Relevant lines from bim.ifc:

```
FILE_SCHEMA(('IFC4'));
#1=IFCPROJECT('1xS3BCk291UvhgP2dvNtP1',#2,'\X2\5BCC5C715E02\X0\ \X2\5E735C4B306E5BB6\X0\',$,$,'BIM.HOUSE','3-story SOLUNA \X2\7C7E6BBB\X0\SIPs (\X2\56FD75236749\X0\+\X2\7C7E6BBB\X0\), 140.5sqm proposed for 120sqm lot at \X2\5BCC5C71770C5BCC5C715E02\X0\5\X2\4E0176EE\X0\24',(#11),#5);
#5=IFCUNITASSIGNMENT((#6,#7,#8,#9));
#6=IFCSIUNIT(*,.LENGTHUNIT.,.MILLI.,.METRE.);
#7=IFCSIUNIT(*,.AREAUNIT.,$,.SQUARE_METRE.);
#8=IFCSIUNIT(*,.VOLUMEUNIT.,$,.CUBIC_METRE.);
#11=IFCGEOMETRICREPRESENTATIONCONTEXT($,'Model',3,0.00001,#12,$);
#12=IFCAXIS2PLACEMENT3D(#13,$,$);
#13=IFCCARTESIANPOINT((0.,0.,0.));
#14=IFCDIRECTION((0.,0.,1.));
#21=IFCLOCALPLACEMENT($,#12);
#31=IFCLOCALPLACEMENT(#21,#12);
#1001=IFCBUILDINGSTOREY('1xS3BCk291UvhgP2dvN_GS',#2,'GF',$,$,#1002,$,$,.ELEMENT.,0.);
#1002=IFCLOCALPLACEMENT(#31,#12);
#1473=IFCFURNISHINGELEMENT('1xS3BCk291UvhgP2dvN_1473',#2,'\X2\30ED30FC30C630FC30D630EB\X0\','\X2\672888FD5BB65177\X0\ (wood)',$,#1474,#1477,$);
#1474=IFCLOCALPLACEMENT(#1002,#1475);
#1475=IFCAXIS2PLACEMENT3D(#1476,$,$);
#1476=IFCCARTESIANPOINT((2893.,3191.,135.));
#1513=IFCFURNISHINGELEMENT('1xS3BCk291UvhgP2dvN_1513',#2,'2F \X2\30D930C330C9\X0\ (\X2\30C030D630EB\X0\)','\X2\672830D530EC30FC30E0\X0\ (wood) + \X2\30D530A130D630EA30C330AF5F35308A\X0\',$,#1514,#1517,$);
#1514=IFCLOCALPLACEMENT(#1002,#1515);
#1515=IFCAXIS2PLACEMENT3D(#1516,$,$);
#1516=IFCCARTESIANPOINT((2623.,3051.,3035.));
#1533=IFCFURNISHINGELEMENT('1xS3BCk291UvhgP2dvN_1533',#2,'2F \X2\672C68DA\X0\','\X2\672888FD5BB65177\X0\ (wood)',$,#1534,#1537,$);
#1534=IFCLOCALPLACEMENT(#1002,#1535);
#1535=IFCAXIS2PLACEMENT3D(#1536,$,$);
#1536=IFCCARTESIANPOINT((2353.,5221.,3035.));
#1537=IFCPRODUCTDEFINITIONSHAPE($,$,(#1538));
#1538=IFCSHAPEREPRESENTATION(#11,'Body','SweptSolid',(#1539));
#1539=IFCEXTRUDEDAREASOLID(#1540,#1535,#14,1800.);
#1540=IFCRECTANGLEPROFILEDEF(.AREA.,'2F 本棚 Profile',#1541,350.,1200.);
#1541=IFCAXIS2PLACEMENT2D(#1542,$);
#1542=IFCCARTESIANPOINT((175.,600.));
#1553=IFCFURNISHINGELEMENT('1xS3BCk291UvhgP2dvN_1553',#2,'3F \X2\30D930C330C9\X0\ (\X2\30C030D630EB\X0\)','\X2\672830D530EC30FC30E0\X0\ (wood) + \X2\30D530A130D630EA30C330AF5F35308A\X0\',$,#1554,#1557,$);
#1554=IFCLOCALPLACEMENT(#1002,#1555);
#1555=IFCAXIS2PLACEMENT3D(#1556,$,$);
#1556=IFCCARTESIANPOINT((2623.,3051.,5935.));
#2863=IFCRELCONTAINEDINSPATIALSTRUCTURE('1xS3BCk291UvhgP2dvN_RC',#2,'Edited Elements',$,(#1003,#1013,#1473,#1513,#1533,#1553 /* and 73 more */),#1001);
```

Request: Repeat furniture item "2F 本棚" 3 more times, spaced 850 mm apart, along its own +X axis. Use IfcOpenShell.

```python
import ifcopenshell
import ifcopenshell.api.geometry
import ifcopenshell.api.root
import ifcopenshell.util.element
import ifcopenshell.util.placement
import ifcopenshell.util.unit

model = ifcopenshell.open("bim.ifc")
unit_scale = ifcopenshell.util.unit.calculate_unit_scale(model)


def reuse_history(source, copy):
    """copy_class also copies each property set's owner history, people and application; keep the originals."""
    for rel in copy.IsDefinedBy:
        if rel.is_a("IfcRelDefinesByProperties") and (history := rel.RelatingPropertyDefinition.OwnerHistory):
            rel.RelatingPropertyDefinition.OwnerHistory = source.OwnerHistory
            ifcopenshell.util.element.remove_deep2(model, history)


source = model.by_id(1533)
base = ifcopenshell.util.placement.get_local_placement(source.ObjectPlacement)
step = base[:3, 0] * 0.85 / unit_scale

for i in range(1, 4):
    copy = ifcopenshell.api.root.copy_class(model, product=source)
    copy.Representation = ifcopenshell.util.element.copy_deep(
        model, source.Representation, exclude=["IfcGeometricRepresentationContext", "IfcRepresentationMap"]
    )
    reuse_history(source, copy)
    matrix = base.copy()
    matrix[:3, 3] += i * step
    print("added at", matrix[:3, 3].round(3) + 0.0)
    ifcopenshell.api.geometry.edit_object_placement(model, product=copy, matrix=matrix, is_si=False)

model.write("bim_v2.ifc")
```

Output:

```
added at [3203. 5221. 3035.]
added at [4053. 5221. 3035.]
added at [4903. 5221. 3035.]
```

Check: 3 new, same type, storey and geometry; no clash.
